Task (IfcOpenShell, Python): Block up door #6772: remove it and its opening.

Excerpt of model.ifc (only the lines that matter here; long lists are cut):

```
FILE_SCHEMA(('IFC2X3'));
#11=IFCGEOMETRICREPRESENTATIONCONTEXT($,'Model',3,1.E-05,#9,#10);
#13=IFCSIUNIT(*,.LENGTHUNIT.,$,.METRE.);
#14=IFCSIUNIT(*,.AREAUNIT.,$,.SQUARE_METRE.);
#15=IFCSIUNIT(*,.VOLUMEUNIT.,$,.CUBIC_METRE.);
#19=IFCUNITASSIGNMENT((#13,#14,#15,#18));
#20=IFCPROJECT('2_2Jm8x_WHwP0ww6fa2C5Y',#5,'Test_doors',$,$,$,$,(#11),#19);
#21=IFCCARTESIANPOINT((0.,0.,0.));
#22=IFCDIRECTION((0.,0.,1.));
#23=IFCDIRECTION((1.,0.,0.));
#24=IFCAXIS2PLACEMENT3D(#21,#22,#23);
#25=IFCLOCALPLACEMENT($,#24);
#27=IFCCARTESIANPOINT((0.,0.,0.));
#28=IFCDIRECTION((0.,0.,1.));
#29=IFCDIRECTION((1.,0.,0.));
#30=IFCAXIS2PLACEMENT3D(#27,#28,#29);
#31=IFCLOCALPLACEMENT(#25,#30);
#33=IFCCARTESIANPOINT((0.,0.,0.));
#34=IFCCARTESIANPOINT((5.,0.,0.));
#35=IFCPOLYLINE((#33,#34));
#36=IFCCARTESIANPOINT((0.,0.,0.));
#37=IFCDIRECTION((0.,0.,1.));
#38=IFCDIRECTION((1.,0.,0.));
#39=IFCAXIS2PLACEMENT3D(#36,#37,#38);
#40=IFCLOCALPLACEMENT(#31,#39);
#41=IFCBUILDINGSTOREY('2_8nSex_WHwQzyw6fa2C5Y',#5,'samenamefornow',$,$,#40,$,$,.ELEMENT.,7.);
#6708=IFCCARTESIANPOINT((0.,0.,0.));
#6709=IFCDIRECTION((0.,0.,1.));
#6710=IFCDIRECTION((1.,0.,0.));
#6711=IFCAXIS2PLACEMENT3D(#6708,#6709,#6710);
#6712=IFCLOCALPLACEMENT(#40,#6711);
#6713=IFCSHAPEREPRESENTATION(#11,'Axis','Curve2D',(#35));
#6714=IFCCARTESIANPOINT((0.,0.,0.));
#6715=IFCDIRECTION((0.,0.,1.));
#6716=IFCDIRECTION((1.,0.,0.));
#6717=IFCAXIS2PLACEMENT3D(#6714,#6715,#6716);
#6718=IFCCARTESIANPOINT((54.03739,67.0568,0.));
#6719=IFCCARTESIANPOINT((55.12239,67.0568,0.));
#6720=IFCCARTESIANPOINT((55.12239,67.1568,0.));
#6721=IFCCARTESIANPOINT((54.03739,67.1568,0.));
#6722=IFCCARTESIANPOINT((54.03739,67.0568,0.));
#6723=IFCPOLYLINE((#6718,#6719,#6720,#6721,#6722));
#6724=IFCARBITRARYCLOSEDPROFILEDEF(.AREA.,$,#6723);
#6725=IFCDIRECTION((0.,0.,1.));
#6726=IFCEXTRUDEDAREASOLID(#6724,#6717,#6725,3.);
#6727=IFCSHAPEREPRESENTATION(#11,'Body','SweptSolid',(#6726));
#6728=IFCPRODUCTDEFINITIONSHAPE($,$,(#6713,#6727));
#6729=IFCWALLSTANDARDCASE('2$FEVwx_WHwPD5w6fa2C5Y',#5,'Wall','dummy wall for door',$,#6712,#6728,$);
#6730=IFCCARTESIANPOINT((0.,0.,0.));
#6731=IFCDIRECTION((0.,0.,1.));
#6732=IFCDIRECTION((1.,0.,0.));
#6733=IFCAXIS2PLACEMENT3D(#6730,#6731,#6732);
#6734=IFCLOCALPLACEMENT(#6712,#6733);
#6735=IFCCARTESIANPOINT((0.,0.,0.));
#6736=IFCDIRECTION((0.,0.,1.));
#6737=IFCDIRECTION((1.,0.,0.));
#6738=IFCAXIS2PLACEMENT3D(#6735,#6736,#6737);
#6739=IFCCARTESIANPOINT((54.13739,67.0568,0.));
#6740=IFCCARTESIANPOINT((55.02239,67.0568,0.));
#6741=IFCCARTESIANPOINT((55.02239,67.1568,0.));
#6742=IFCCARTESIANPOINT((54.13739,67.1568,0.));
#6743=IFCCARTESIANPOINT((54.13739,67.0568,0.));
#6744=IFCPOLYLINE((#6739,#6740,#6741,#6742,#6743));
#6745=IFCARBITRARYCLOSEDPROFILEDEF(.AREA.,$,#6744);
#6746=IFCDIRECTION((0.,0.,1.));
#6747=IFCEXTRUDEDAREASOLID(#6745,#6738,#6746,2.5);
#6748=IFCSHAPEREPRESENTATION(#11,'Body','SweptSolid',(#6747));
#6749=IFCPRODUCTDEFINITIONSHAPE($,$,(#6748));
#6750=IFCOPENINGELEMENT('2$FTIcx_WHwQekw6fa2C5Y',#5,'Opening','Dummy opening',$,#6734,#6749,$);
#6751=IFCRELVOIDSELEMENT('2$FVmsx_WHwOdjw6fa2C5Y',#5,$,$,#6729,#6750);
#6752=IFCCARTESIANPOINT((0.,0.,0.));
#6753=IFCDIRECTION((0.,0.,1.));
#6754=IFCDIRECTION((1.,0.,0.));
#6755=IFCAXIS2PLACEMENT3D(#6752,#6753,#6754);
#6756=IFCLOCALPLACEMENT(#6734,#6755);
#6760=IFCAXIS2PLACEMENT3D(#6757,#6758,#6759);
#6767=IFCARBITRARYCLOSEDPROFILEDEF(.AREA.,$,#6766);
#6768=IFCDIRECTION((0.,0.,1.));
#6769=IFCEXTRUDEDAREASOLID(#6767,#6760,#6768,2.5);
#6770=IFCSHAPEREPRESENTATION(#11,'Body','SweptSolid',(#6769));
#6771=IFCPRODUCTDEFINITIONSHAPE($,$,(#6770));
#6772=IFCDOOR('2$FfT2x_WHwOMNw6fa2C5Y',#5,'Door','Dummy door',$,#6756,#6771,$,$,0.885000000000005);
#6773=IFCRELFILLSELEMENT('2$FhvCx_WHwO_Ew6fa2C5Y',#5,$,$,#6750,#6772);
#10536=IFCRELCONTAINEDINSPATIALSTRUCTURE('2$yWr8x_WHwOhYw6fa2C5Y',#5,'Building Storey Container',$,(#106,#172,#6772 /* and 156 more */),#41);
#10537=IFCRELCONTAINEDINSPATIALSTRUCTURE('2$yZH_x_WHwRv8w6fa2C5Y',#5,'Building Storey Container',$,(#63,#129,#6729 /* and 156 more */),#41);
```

```python
import ifcopenshell
import ifcopenshell.api.feature
import ifcopenshell.api.root
import ifcopenshell.geom
import ifcopenshell.util.shape

model = ifcopenshell.open("model.ifc")
settings = ifcopenshell.geom.settings()


def volume(element):
    """Net volume in cubic metres, openings subtracted."""
    shape = ifcopenshell.geom.create_shape(settings, element)
    return ifcopenshell.util.shape.get_volume(shape.geometry)


door = model.by_guid("2$FfT2x_WHwOMNw6fa2C5Y")
opening = door.FillsVoids[0].RelatingOpeningElement
wall = opening.VoidsElements[0].RelatingBuildingElement
before = volume(wall)

ifcopenshell.api.root.remove_product(model, product=door)
ifcopenshell.api.feature.remove_feature(model, feature=opening)

after = volume(wall)

print(f"wall volume {before:.3f} -> {after:.3f} m3")

model.write("model_v2.ifc")
```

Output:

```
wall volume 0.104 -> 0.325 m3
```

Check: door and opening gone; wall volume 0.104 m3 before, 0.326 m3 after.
